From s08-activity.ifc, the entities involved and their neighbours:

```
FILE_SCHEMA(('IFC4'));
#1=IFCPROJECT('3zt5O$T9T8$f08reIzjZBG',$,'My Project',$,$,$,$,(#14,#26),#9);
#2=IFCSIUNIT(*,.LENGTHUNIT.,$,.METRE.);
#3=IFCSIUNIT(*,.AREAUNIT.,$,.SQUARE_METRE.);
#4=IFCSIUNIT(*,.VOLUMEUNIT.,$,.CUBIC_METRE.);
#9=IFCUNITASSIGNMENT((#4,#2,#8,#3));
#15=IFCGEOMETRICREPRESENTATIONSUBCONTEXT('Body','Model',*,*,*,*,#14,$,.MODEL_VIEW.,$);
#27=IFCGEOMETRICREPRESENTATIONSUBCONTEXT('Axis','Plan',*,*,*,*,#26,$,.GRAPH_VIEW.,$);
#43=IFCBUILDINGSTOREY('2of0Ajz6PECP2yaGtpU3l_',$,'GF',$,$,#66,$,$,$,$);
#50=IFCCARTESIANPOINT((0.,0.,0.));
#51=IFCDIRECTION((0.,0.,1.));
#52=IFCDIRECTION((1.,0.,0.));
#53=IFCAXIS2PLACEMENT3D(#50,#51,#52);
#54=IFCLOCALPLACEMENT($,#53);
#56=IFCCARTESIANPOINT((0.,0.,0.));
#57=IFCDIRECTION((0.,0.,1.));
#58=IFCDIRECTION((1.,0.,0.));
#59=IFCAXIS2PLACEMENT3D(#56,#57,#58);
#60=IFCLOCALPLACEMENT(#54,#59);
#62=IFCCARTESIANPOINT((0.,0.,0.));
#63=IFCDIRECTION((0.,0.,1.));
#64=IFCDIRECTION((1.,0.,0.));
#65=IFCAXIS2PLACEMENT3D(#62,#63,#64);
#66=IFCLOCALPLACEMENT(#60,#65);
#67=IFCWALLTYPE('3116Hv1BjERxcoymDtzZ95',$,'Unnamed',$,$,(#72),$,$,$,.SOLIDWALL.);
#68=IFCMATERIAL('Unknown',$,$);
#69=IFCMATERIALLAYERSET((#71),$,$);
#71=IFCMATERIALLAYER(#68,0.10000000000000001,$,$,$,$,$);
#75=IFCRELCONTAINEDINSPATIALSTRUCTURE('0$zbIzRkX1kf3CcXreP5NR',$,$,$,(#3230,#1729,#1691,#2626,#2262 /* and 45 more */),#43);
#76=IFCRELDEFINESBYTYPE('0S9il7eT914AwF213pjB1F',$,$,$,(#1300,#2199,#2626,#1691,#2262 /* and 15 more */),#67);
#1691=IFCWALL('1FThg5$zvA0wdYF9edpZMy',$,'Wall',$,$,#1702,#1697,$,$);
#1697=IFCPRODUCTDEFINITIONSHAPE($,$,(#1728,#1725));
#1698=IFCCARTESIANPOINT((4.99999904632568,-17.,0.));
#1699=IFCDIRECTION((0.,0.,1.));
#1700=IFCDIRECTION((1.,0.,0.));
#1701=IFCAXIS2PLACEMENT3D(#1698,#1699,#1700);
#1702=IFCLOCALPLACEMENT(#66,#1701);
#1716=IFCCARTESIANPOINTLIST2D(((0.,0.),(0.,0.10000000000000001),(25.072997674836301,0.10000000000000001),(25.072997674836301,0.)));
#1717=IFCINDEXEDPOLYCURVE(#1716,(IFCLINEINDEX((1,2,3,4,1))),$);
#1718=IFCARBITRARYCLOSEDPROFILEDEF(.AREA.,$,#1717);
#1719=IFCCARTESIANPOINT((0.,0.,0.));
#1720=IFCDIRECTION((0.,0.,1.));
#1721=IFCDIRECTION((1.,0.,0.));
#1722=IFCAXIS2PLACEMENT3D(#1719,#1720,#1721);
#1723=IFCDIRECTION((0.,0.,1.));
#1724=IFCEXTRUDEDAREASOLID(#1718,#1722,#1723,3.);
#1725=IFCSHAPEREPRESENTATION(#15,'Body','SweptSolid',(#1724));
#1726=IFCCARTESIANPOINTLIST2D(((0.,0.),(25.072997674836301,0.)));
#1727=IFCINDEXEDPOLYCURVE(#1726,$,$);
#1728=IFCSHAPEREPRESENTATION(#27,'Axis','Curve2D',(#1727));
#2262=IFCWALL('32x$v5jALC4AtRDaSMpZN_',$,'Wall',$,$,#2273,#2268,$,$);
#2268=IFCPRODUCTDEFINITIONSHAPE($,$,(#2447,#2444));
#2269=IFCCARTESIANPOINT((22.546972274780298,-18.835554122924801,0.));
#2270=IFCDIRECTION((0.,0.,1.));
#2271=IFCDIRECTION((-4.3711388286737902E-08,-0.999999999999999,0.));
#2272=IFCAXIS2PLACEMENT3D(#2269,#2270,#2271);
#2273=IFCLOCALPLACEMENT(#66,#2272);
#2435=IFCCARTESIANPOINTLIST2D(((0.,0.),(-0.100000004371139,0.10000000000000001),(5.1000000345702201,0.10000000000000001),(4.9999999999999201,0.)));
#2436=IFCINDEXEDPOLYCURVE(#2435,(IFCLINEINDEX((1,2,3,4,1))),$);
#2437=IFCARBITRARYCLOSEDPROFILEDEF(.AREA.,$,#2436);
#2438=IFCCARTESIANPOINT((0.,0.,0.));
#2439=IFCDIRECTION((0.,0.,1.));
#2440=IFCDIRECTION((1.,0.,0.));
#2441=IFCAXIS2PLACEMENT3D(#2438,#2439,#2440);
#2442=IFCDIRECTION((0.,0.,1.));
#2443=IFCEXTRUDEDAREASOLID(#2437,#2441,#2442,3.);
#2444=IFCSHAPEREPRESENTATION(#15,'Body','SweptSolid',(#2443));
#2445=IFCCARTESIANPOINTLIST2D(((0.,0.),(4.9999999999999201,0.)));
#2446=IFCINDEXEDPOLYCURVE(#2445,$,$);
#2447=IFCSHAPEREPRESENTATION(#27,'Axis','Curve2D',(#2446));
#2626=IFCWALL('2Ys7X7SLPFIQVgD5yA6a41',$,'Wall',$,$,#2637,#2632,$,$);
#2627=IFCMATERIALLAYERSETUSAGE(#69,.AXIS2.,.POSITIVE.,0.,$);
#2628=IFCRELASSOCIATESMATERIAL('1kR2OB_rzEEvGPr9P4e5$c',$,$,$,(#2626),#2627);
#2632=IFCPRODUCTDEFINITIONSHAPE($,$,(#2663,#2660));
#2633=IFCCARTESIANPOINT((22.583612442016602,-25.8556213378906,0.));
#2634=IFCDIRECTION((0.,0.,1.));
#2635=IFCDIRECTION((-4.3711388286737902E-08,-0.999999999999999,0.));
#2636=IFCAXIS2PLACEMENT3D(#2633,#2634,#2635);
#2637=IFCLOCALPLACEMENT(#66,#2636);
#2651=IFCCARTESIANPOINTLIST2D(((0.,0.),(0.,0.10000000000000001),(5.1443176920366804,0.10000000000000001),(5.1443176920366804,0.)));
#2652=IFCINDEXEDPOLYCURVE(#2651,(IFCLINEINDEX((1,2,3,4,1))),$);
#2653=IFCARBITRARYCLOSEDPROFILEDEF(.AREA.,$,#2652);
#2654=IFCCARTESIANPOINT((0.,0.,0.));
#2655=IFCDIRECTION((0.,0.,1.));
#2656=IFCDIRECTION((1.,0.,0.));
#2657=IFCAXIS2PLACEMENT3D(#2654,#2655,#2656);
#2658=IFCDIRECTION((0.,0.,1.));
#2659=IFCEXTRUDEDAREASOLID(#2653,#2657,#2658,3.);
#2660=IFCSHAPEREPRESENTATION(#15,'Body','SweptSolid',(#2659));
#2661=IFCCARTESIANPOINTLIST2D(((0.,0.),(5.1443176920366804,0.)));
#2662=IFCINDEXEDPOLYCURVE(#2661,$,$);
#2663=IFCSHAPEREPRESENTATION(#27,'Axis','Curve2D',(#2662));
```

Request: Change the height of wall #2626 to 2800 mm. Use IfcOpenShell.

```python
import ifcopenshell
import ifcopenshell.geom
import ifcopenshell.util.representation
import ifcopenshell.util.shape
import ifcopenshell.util.unit

model = ifcopenshell.open("s08-activity.ifc")
unit_scale = ifcopenshell.util.unit.calculate_unit_scale(model)
settings = ifcopenshell.geom.settings()


def volume(element):
    """Net volume in cubic metres, openings subtracted."""
    shape = ifcopenshell.geom.create_shape(settings, element)
    return ifcopenshell.util.shape.get_volume(shape.geometry)


wall = model.by_guid("2Ys7X7SLPFIQVgD5yA6a41")
before = volume(wall)

body = ifcopenshell.util.representation.get_representation(wall, "Model", "Body")
solid = body.Items[0]
old_height = solid.Depth
solid.Depth = 2.8 / unit_scale
after = volume(wall)

print(f"height {old_height:g} -> {solid.Depth:g}, volume {before:.3f} -> {after:.3f} m3")

model.write("s08-activity_updated.ifc")
```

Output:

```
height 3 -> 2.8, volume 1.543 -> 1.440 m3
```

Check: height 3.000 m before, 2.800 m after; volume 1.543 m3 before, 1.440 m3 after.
